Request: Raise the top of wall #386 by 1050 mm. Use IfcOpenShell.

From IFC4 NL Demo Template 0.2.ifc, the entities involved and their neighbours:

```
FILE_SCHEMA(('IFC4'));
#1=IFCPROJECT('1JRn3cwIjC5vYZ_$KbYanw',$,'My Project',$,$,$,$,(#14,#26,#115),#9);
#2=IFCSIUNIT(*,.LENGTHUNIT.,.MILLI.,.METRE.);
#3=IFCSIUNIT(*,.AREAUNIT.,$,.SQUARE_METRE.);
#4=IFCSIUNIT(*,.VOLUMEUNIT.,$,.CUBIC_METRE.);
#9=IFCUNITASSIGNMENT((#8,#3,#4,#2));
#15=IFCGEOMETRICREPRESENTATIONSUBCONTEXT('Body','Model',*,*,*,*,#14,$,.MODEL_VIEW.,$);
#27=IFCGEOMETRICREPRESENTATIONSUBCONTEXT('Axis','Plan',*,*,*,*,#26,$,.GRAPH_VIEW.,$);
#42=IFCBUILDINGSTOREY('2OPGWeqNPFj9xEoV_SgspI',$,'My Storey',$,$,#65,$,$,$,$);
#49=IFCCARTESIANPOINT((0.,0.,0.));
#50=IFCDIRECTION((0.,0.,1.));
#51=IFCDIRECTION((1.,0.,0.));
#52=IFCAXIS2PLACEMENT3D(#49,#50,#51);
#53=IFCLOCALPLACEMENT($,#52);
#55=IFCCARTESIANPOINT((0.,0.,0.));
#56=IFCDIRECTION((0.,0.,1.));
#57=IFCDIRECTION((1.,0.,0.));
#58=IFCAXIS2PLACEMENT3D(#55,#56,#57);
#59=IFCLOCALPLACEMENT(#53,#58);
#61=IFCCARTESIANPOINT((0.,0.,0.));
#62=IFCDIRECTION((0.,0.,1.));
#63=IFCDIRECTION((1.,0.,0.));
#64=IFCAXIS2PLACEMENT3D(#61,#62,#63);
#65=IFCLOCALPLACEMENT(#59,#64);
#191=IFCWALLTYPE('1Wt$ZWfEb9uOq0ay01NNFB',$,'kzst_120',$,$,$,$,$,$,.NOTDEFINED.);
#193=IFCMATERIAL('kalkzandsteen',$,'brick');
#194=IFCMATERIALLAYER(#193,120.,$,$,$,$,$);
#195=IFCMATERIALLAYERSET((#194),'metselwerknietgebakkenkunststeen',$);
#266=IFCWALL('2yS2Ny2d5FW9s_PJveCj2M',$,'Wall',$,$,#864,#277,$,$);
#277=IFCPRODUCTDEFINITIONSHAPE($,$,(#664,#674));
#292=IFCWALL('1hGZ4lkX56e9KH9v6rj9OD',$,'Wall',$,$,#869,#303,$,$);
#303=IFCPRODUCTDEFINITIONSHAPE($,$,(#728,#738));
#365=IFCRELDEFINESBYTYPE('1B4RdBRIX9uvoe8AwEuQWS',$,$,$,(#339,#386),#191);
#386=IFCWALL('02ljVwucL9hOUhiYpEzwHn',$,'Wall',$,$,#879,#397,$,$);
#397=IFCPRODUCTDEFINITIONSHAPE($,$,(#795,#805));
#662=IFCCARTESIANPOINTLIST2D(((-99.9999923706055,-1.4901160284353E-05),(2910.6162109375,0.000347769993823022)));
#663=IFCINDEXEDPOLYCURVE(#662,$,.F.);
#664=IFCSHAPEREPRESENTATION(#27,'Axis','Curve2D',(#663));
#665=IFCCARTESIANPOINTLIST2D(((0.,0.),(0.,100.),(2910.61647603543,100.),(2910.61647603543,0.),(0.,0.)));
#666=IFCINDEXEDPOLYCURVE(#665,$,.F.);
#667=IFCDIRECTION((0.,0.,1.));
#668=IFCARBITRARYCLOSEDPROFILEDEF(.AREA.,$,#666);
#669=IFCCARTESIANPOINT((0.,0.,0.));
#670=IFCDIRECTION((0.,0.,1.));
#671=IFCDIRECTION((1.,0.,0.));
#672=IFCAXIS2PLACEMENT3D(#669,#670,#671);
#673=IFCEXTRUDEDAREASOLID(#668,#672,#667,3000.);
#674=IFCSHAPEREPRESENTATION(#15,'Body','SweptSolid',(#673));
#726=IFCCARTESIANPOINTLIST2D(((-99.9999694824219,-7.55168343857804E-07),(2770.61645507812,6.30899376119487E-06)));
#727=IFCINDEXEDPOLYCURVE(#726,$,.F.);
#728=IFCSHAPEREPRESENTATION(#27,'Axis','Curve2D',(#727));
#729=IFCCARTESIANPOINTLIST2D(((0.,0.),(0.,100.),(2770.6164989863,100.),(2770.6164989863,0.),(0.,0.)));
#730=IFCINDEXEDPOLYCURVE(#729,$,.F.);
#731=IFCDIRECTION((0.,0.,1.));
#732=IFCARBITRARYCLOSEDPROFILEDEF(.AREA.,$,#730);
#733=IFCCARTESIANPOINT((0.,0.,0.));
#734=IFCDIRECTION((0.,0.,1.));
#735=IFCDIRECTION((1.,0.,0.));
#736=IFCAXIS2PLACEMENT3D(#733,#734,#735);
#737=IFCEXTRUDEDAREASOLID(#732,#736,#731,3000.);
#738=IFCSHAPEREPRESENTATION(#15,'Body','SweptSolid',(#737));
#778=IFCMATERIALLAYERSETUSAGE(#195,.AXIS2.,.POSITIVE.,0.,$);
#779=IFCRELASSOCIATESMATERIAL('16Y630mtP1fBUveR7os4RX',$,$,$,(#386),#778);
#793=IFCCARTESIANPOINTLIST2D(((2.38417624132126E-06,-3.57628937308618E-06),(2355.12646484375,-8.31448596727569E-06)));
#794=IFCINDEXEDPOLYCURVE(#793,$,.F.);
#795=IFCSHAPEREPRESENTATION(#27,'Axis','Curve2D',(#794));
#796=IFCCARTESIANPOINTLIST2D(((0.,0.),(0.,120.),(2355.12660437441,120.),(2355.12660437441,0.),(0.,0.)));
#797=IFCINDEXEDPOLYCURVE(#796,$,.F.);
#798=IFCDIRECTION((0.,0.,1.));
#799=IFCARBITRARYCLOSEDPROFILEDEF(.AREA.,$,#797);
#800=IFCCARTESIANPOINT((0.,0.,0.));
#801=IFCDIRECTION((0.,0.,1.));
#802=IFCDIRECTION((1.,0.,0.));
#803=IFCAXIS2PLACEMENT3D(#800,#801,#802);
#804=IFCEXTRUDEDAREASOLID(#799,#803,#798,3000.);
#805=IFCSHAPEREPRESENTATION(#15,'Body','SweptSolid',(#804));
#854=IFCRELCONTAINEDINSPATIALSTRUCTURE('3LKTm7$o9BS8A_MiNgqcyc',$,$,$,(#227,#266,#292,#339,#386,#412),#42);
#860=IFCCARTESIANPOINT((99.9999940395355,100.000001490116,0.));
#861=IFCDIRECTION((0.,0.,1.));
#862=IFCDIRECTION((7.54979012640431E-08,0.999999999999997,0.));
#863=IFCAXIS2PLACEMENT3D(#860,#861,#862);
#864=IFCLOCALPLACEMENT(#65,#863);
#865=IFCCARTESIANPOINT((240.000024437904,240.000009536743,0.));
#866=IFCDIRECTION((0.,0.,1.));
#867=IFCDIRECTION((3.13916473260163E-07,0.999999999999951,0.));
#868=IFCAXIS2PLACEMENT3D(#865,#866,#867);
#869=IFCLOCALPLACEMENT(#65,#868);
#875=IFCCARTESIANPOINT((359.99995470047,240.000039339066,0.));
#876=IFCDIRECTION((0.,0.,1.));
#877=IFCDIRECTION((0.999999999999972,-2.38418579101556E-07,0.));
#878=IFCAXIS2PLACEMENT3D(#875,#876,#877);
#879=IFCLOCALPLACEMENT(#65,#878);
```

```python
import ifcopenshell
import ifcopenshell.geom
import ifcopenshell.util.representation
import ifcopenshell.util.shape
import ifcopenshell.util.unit

model = ifcopenshell.open("IFC4 NL Demo Template 0.2.ifc")
unit_scale = ifcopenshell.util.unit.calculate_unit_scale(model)
settings = ifcopenshell.geom.settings()


def volume(element):
    """Net volume in cubic metres, openings subtracted."""
    shape = ifcopenshell.geom.create_shape(settings, element)
    return ifcopenshell.util.shape.get_volume(shape.geometry)


wall = model.by_guid("02ljVwucL9hOUhiYpEzwHn")
before = volume(wall)

body = ifcopenshell.util.representation.get_representation(wall, "Model", "Body")
solid = body.Items[0]
old_height = solid.Depth
solid.Depth += 1.05 / unit_scale
after = volume(wall)

print(f"height {old_height:g} -> {solid.Depth:g}, volume {before:.3f} -> {after:.3f} m3")

model.write("IFC4 NL Demo Template 0.2_updated.ifc")
```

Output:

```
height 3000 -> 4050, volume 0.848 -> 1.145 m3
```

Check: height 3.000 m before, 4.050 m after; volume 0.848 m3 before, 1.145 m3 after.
